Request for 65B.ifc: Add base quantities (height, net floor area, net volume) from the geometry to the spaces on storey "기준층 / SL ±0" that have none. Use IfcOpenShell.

First a look at what the model holds.

```python
import ifcopenshell
import ifcopenshell.util.element
import ifcopenshell.util.unit

model = ifcopenshell.open("65B.ifc")
print(model.schema)
for unit_type in ("LENGTHUNIT", "AREAUNIT", "VOLUMEUNIT"):
    print(unit_type, ifcopenshell.util.unit.calculate_unit_scale(model, unit_type))
storey = next(s for s in model.by_type("IfcBuildingStorey") if s.Name == "기준층 / SL ±0")
spaces = [e for e in ifcopenshell.util.element.get_decomposition(storey) if e.is_a("IfcSpace")]
for e in sorted(spaces, key=lambda e: e.id()):
    print(e.id(), e.is_a(), e.Name, list(ifcopenshell.util.element.get_psets(e, qtos_only=True)), sep=" | ")
```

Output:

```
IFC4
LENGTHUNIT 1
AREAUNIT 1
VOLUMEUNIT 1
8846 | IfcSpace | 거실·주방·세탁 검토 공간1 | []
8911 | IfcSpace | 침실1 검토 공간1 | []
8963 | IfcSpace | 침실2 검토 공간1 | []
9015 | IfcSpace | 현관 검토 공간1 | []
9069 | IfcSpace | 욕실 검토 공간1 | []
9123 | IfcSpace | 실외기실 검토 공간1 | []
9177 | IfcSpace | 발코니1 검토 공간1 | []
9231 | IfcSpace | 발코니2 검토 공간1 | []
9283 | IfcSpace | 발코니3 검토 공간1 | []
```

```python
import ifcopenshell
import ifcopenshell.api.pset
import ifcopenshell.geom
import ifcopenshell.util.element
import ifcopenshell.util.shape
import ifcopenshell.util.unit

model = ifcopenshell.open("65B.ifc")
unit_scale = ifcopenshell.util.unit.calculate_unit_scale(model)
area_scale = ifcopenshell.util.unit.calculate_unit_scale(model, "AREAUNIT")
volume_scale = ifcopenshell.util.unit.calculate_unit_scale(model, "VOLUMEUNIT")
settings = ifcopenshell.geom.settings()

storey = next(s for s in model.by_type("IfcBuildingStorey") if s.Name == "기준층 / SL ±0")
spaces = [e for e in ifcopenshell.util.element.get_decomposition(storey) if e.is_a("IfcSpace")]

for e in sorted(spaces, key=lambda e: e.id()):
    if ifcopenshell.util.element.get_psets(e, qtos_only=True, should_inherit=False):
        continue
    # Geometry comes back in metres, in the element's own axes.
    shape = ifcopenshell.geom.create_shape(settings, e)
    values = {
        "Height": ifcopenshell.util.shape.get_z(shape.geometry) / unit_scale,
        "NetFloorArea": ifcopenshell.util.shape.get_footprint_area(shape.geometry) / area_scale,
        "NetVolume": ifcopenshell.util.shape.get_volume(shape.geometry) / volume_scale,
    }
    qto = ifcopenshell.api.pset.add_qto(model, product=e, name="Qto_SpaceBaseQuantities")
    ifcopenshell.api.pset.edit_qto(model, qto=qto, properties=values)
    print(e.id(), {k: round(v, 3) for k, v in values.items()})

model.write("65B_rev.ifc")
```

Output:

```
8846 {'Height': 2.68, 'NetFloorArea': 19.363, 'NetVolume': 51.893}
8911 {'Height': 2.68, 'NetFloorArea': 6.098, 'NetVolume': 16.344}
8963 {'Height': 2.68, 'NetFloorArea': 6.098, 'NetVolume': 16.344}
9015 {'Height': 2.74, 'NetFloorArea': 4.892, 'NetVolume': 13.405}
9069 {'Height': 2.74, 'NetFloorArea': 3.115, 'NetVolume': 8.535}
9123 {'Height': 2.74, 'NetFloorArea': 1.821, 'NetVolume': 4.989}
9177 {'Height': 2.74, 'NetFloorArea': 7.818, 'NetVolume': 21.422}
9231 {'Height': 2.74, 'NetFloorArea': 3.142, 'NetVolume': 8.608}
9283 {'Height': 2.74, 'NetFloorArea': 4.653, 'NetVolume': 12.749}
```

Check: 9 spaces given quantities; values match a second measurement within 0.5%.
